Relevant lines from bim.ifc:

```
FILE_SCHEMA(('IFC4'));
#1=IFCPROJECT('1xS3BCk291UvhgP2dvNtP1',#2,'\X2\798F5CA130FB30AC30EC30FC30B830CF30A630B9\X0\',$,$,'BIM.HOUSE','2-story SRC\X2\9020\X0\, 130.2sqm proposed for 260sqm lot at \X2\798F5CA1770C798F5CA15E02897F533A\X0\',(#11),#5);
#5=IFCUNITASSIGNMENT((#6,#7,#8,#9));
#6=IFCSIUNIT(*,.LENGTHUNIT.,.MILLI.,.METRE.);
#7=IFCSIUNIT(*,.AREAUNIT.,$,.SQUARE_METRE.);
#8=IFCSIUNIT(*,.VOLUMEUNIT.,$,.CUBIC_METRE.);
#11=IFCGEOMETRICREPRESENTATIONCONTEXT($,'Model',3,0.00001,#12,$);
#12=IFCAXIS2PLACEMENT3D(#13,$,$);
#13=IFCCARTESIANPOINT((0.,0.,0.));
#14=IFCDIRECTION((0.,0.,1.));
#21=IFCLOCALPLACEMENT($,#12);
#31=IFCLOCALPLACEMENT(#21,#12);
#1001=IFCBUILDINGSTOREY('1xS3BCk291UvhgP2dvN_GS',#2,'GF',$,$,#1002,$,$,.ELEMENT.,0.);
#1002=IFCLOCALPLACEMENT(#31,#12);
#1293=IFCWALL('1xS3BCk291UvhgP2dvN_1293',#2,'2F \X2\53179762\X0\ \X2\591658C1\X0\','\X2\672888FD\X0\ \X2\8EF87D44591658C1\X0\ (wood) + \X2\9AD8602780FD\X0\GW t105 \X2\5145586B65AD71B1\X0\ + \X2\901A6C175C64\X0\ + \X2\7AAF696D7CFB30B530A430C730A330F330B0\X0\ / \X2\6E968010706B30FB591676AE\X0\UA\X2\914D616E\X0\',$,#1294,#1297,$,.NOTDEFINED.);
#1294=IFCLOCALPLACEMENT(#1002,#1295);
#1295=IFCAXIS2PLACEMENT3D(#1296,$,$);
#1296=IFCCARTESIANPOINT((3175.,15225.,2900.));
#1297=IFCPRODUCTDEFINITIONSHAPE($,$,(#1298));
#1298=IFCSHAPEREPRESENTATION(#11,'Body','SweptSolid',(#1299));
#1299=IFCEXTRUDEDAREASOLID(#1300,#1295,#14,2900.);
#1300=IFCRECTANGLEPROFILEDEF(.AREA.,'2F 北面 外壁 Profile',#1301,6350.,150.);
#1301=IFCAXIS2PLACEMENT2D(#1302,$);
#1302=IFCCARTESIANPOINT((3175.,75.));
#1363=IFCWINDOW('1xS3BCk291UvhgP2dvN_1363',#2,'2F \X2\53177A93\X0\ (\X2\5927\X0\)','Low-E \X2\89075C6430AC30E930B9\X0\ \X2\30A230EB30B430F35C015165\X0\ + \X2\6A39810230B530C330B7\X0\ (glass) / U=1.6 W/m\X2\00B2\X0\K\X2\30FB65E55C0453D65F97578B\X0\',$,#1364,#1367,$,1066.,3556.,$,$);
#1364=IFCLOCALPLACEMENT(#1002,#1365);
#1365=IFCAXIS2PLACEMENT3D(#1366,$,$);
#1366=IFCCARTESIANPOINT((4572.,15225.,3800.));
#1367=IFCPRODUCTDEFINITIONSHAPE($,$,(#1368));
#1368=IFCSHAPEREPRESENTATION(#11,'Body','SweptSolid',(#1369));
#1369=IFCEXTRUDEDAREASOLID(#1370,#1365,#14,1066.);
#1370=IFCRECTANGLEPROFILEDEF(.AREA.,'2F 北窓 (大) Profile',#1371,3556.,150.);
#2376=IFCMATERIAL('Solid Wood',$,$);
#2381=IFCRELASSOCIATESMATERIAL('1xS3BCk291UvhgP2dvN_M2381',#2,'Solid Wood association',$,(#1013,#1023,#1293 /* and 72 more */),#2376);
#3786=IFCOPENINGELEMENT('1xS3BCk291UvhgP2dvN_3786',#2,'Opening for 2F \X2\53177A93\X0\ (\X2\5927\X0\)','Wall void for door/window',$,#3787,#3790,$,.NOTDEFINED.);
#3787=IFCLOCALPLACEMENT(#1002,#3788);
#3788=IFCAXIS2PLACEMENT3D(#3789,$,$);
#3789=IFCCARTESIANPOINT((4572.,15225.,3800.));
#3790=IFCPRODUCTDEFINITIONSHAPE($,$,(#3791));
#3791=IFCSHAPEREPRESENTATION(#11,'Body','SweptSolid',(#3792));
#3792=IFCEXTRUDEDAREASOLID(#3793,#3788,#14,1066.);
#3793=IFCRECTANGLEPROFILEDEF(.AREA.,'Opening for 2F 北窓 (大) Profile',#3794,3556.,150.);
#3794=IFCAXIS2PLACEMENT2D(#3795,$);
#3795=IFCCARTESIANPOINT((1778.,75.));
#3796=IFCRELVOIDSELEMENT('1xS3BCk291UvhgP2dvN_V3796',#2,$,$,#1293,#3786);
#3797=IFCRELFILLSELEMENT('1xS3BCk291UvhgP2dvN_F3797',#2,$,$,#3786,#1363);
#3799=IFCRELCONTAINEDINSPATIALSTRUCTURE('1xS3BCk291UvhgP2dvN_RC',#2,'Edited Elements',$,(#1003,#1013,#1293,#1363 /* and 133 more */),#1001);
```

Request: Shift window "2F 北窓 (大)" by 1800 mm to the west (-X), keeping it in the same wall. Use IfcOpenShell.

```python
import ifcopenshell
import ifcopenshell.api.geometry
import ifcopenshell.util.placement
import ifcopenshell.util.unit

model = ifcopenshell.open("bim.ifc")
unit_scale = ifcopenshell.util.unit.calculate_unit_scale(model)

window = model.by_guid("1xS3BCk291UvhgP2dvN_1363")
opening = window.FillsVoids[0].RelatingOpeningElement
wall = opening.VoidsElements[0].RelatingBuildingElement

wall_matrix = ifcopenshell.util.placement.get_local_placement(wall.ObjectPlacement)
shift = wall_matrix[:3, 0] * -1.8 / unit_scale
before = ifcopenshell.util.placement.get_local_placement(window.ObjectPlacement)[:3, 3].copy()

# The window is not placed relative to its opening, so move both.
for product in (opening, window):
    matrix = ifcopenshell.util.placement.get_local_placement(product.ObjectPlacement)
    matrix[:3, 3] += shift
    ifcopenshell.api.geometry.edit_object_placement(model, product=product, matrix=matrix, is_si=False)

after = ifcopenshell.util.placement.get_local_placement(window.ObjectPlacement)[:3, 3]
print("window moved by", (after - before).round(3) + 0.0)

model.write("bim-out.ifc")
```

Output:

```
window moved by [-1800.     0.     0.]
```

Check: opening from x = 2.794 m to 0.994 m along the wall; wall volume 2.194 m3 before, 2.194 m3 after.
